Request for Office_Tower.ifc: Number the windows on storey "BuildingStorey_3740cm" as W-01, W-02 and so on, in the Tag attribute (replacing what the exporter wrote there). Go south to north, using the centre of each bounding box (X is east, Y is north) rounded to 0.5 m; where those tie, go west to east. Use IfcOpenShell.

First a look at what the model holds.

```python
import ifcopenshell
import ifcopenshell.util.element
import ifcopenshell.util.placement

model = ifcopenshell.open("Office_Tower.ifc")
print(model.schema)
storey = next(s for s in model.by_type("IfcBuildingStorey") if s.Name == "BuildingStorey_3740cm")
windows = [e for e in ifcopenshell.util.element.get_decomposition(storey) if e.is_a("IfcWindow")]
for e in sorted(windows, key=lambda e: e.id()):
    origin = ifcopenshell.util.placement.get_local_placement(e.ObjectPlacement)[:3, 3]
    print(e.id(), e.Tag, e.Name, origin.round(2) + 0.0, sep=" | ")
```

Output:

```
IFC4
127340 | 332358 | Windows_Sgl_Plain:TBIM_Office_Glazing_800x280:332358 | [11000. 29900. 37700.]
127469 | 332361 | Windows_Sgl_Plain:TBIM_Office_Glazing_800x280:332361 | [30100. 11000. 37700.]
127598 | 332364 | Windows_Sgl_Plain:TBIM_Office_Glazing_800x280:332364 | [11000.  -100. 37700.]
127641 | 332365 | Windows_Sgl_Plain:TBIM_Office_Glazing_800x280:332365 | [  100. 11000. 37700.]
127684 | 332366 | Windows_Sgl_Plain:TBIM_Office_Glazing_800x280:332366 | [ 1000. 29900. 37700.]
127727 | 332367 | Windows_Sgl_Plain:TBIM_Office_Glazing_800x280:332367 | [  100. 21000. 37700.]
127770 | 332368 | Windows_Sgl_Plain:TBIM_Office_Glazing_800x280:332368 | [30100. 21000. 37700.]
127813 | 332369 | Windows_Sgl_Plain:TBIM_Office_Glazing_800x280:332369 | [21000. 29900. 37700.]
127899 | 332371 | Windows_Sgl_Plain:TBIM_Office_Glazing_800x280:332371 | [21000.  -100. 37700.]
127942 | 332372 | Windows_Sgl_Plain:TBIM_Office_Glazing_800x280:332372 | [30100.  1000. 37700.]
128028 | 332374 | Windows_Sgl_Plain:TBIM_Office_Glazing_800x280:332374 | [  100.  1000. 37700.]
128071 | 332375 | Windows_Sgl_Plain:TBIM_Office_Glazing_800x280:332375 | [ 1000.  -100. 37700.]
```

```python
import ifcopenshell
import ifcopenshell.geom
import ifcopenshell.util.element
import ifcopenshell.util.shape

model = ifcopenshell.open("Office_Tower.ifc")
settings = ifcopenshell.geom.settings()
settings.set("use-world-coords", True)


def centre(element):
    shape = ifcopenshell.geom.create_shape(settings, element)
    return ifcopenshell.util.shape.get_bbox_centroid(shape.geometry)


storey = next(s for s in model.by_type("IfcBuildingStorey") if s.Name == "BuildingStorey_3740cm")
windows = [e for e in ifcopenshell.util.element.get_decomposition(storey) if e.is_a("IfcWindow")]

# Insertion points can sit at a corner or the storey origin, so sort by the geometry (in metres).
centres = {e: centre(e) for e in windows}
windows.sort(key=lambda e: (round(centres[e][1] / 0.5), centres[e][0]))

for i, e in enumerate(windows, start=1):
    number = f"W-{i:02d}"
    e.Tag = number
    print(e.id(), number)

model.write("Office_Tower-out.ifc")
```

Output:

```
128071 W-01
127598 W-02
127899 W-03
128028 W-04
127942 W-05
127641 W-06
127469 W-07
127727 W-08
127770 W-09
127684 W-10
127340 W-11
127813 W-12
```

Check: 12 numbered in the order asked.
